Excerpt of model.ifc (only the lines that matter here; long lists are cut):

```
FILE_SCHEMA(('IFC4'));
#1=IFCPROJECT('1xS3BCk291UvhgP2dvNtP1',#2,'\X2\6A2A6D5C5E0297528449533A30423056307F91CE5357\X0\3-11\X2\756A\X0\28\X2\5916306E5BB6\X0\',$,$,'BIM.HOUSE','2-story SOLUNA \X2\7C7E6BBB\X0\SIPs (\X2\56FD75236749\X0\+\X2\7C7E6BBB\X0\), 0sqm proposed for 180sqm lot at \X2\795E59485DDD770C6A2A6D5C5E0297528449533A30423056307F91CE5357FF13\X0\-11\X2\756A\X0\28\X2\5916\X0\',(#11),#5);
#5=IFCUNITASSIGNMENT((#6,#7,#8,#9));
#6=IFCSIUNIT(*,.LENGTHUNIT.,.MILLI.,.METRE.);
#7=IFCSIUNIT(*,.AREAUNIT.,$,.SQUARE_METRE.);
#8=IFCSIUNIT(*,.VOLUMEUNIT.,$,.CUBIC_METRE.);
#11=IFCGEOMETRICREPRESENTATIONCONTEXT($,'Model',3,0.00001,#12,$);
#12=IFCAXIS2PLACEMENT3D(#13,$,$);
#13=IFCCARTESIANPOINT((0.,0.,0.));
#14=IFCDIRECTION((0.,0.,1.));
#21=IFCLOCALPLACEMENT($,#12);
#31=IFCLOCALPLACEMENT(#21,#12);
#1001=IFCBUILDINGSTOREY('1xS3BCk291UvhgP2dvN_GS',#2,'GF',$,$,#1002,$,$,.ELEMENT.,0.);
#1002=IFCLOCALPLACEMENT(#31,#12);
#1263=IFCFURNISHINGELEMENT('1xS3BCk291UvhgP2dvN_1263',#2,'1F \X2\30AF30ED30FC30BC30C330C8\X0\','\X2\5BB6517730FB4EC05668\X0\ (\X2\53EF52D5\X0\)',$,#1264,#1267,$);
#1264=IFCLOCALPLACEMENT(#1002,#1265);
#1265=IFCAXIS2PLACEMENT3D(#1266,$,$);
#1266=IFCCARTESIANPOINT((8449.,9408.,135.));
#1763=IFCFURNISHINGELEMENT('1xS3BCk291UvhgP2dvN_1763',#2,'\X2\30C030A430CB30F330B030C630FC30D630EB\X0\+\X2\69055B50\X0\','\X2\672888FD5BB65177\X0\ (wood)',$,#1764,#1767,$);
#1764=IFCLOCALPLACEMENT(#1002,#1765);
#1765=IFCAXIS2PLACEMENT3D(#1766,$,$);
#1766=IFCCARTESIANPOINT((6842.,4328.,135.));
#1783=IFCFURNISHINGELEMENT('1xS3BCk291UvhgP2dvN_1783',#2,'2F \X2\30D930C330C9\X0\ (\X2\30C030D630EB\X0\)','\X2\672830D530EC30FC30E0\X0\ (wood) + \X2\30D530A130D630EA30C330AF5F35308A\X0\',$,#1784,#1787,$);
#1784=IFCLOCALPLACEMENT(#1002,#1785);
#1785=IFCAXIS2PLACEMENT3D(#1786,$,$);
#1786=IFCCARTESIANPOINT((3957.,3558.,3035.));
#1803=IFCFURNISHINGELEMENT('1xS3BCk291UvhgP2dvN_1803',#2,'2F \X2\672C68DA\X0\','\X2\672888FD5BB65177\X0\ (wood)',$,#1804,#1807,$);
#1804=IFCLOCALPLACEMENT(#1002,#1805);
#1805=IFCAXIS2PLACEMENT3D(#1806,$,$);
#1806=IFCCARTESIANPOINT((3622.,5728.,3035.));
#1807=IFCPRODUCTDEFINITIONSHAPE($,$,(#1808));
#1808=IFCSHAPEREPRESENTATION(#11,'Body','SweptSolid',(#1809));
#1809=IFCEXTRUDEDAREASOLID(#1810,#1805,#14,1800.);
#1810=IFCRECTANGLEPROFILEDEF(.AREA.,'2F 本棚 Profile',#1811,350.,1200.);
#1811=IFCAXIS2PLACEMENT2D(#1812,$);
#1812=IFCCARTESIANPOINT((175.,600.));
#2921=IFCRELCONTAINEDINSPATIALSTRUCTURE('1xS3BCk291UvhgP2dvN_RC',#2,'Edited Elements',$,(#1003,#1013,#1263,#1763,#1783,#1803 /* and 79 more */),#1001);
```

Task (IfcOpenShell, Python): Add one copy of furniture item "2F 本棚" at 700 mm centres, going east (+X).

```python
import numpy as np
import ifcopenshell
import ifcopenshell.api.geometry
import ifcopenshell.api.root
import ifcopenshell.util.element
import ifcopenshell.util.placement
import ifcopenshell.util.unit

model = ifcopenshell.open("model.ifc")
unit_scale = ifcopenshell.util.unit.calculate_unit_scale(model)


def reuse_history(source, copy):
    """copy_class also copies each property set's owner history, people and application; keep the originals."""
    for rel in copy.IsDefinedBy:
        if rel.is_a("IfcRelDefinesByProperties") and (history := rel.RelatingPropertyDefinition.OwnerHistory):
            rel.RelatingPropertyDefinition.OwnerHistory = source.OwnerHistory
            ifcopenshell.util.element.remove_deep2(model, history)


source = model.by_id(1803)
base = ifcopenshell.util.placement.get_local_placement(source.ObjectPlacement)
step = np.array([1.0, 0.0, 0.0]) * 0.7 / unit_scale

for i in range(1, 2):
    copy = ifcopenshell.api.root.copy_class(model, product=source)
    copy.Representation = ifcopenshell.util.element.copy_deep(
        model, source.Representation, exclude=["IfcGeometricRepresentationContext", "IfcRepresentationMap"]
    )
    reuse_history(source, copy)
    matrix = base.copy()
    matrix[:3, 3] += i * step
    print("added at", matrix[:3, 3].round(3) + 0.0)
    ifcopenshell.api.geometry.edit_object_placement(model, product=copy, matrix=matrix, is_si=False)

model.write("model_rev.ifc")
```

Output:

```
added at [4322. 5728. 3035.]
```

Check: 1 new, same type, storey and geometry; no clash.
